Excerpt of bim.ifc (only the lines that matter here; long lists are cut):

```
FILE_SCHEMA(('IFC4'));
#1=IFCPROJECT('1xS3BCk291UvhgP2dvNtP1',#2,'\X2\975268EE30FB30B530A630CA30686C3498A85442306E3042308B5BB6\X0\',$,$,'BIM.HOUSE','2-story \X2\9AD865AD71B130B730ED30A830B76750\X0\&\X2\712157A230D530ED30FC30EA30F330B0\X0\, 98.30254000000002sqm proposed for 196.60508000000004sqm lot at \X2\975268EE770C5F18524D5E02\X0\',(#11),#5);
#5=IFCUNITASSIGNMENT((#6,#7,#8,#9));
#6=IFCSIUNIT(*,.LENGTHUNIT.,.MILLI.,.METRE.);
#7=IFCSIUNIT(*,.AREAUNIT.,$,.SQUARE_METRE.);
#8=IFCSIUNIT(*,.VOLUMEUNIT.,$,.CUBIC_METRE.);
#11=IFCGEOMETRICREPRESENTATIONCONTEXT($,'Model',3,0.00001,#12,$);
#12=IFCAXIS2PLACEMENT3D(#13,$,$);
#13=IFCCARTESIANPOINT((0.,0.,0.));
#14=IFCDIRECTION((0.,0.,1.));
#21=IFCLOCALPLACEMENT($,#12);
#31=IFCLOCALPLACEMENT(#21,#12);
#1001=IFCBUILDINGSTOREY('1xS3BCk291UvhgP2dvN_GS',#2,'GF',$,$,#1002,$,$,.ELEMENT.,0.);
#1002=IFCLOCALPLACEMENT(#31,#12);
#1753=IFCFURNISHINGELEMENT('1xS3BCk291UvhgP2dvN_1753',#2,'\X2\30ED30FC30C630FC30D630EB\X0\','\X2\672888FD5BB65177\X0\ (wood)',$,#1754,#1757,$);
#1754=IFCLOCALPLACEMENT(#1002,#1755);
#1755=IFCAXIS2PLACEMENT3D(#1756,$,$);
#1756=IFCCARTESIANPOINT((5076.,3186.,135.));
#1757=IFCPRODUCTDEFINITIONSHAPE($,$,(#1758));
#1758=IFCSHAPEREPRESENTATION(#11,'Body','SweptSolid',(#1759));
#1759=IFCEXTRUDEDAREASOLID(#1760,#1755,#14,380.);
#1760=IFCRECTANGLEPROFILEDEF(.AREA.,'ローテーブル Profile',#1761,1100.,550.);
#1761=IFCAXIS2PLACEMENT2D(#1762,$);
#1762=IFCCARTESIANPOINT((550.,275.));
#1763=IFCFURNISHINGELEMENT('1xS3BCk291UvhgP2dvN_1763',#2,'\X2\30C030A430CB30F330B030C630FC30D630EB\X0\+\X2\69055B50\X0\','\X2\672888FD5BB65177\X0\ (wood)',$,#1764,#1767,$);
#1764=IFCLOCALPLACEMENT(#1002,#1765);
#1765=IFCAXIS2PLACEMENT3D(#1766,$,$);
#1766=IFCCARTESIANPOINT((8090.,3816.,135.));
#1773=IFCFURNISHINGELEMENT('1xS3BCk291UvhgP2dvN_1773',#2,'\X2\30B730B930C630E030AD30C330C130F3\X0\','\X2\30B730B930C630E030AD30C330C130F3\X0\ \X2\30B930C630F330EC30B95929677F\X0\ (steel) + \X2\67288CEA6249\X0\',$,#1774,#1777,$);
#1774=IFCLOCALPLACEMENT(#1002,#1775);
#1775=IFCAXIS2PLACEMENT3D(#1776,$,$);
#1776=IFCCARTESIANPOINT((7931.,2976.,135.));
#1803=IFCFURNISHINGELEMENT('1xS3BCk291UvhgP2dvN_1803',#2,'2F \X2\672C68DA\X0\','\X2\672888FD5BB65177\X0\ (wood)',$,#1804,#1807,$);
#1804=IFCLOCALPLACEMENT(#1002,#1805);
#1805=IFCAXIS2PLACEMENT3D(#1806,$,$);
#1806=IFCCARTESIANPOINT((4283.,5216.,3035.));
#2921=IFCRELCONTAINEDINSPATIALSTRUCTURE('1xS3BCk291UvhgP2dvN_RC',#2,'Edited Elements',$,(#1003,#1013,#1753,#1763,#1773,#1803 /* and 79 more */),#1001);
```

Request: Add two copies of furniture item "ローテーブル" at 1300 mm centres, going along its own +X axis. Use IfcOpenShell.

```python
import ifcopenshell
import ifcopenshell.api.geometry
import ifcopenshell.api.root
import ifcopenshell.util.element
import ifcopenshell.util.placement
import ifcopenshell.util.unit

model = ifcopenshell.open("bim.ifc")
unit_scale = ifcopenshell.util.unit.calculate_unit_scale(model)


def reuse_history(source, copy):
    """copy_class also copies each property set's owner history, people and application; keep the originals."""
    for rel in copy.IsDefinedBy:
        if rel.is_a("IfcRelDefinesByProperties") and (history := rel.RelatingPropertyDefinition.OwnerHistory):
            rel.RelatingPropertyDefinition.OwnerHistory = source.OwnerHistory
            ifcopenshell.util.element.remove_deep2(model, history)


source = model.by_id(1753)
base = ifcopenshell.util.placement.get_local_placement(source.ObjectPlacement)
step = base[:3, 0] * 1.3 / unit_scale

for i in range(1, 3):
    copy = ifcopenshell.api.root.copy_class(model, product=source)
    copy.Representation = ifcopenshell.util.element.copy_deep(
        model, source.Representation, exclude=["IfcGeometricRepresentationContext", "IfcRepresentationMap"]
    )
    reuse_history(source, copy)
    matrix = base.copy()
    matrix[:3, 3] += i * step
    print("added at", matrix[:3, 3].round(3) + 0.0)
    ifcopenshell.api.geometry.edit_object_placement(model, product=copy, matrix=matrix, is_si=False)

model.write("bim_updated.ifc")
```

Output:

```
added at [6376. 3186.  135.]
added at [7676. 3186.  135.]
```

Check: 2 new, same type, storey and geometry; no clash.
